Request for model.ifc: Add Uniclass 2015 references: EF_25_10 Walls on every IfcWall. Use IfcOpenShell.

First a look at what the model holds.

```python
import ifcopenshell

model = ifcopenshell.open("model.ifc")
print(model.schema)
print("classifications:", [c.Name for c in model.by_type("IfcClassification")])
for ifc_class in ("IfcDoor", "IfcRoof", "IfcStair", "IfcWall", "IfcWindow"):
    print(ifc_class, len(model.by_type(ifc_class)))
```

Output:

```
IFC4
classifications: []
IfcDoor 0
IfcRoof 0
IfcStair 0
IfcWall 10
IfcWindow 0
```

```python
import ifcopenshell
import ifcopenshell.api.classification

model = ifcopenshell.open("model.ifc")

system = ifcopenshell.api.classification.add_classification(model, classification="Uniclass 2015")

codes = {
    "IfcWall": ("EF_25_10", "Walls"),
}
for ifc_class, (code, name) in codes.items():
    products = model.by_type(ifc_class)
    ifcopenshell.api.classification.add_reference(
        model, products=products, classification=system, identification=code, name=name
    )
    print(code, len(products))

model.write("model-out.ifc")
```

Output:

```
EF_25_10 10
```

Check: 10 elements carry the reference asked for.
